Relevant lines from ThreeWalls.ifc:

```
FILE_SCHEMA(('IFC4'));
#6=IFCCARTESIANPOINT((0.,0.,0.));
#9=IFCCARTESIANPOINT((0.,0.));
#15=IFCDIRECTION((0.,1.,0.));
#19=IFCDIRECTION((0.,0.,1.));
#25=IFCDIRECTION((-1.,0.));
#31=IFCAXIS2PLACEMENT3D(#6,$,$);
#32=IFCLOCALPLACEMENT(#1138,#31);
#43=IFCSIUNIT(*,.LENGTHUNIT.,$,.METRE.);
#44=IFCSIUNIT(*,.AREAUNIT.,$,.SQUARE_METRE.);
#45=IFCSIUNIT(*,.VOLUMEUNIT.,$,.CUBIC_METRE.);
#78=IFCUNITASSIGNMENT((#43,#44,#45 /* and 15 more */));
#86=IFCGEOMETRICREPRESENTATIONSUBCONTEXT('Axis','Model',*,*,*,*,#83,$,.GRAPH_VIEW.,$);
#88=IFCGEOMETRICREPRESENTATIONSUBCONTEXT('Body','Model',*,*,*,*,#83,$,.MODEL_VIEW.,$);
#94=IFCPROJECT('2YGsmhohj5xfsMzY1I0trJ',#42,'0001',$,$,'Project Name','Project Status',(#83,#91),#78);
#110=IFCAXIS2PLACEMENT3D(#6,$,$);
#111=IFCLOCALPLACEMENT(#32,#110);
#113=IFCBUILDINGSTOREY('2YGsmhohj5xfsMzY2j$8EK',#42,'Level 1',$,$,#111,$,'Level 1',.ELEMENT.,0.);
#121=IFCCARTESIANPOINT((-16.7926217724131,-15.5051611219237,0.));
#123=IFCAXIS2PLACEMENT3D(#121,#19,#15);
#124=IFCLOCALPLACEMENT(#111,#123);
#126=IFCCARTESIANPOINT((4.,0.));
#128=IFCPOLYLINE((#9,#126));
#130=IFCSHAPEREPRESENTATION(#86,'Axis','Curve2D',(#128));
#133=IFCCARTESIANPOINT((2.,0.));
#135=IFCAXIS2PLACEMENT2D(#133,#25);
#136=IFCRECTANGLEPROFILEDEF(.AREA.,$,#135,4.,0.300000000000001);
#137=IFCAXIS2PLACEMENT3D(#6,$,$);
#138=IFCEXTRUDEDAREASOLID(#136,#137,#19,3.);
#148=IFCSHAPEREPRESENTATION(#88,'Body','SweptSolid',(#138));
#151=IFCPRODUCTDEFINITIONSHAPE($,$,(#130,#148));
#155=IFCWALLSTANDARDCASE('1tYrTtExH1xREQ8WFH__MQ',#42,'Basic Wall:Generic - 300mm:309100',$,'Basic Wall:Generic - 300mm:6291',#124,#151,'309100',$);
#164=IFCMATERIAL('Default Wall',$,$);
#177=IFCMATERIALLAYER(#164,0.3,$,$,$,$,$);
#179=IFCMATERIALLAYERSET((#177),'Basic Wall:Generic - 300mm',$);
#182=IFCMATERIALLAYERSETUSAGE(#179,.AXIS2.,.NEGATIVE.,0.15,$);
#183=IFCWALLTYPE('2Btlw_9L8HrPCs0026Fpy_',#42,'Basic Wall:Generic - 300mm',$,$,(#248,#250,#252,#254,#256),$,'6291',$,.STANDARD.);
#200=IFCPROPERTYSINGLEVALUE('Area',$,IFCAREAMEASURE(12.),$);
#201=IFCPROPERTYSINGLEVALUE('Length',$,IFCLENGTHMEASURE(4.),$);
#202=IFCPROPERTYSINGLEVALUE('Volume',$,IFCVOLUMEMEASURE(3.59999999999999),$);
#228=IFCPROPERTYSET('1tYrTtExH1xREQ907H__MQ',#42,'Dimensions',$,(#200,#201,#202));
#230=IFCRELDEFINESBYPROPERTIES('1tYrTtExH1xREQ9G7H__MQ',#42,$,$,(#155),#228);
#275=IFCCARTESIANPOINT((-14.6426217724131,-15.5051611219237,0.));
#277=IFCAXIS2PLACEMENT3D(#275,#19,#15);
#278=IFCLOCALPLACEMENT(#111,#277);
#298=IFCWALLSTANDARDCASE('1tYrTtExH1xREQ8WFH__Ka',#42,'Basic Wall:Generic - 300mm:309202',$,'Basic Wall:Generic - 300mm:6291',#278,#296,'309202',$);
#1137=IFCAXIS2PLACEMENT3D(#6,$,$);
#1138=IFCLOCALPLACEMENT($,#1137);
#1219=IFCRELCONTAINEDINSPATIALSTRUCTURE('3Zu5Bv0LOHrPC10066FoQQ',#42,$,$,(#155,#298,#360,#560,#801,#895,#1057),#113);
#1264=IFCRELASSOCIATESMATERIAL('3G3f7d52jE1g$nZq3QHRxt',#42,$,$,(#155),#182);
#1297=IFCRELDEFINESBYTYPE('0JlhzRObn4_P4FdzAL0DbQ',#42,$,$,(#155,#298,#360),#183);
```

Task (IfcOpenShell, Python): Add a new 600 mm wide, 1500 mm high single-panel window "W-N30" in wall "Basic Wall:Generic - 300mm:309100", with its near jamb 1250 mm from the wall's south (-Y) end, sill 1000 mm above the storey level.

```python
import numpy as np
import ifcopenshell
import ifcopenshell.api.feature
import ifcopenshell.api.geometry
import ifcopenshell.api.pset
import ifcopenshell.api.root
import ifcopenshell.api.spatial
import ifcopenshell.geom
import ifcopenshell.util.element
import ifcopenshell.util.placement
import ifcopenshell.util.representation
import ifcopenshell.util.shape
import ifcopenshell.util.unit

model = ifcopenshell.open("ThreeWalls.ifc")
unit_scale = ifcopenshell.util.unit.calculate_unit_scale(model)
area_scale = ifcopenshell.util.unit.calculate_unit_scale(model, "AREAUNIT")
volume_scale = ifcopenshell.util.unit.calculate_unit_scale(model, "VOLUMEUNIT")
settings = ifcopenshell.geom.settings()


def volume(element):
    """Net volume in cubic metres, openings subtracted."""
    shape = ifcopenshell.geom.create_shape(settings, element)
    return ifcopenshell.util.shape.get_volume(shape.geometry)


wall = model.by_guid("1tYrTtExH1xREQ8WFH__MQ")
storey = ifcopenshell.util.element.get_container(wall, ifc_class="IfcBuildingStorey")
context = ifcopenshell.util.representation.get_context(model, "Model", "Body", "MODEL_VIEW")
before = volume(wall)

width, height, from_end, sill = 0.6, 1.5, 1.25, 1  # metres

# The wall runs along its own X axis, and the end named is its -X end.
wall_shape = ifcopenshell.geom.create_shape(settings, wall)
x, y, z = ifcopenshell.util.shape.get_vertices(wall_shape.geometry).T
start = x.min() + from_end
face, thickness = float(y.min()), float(y.max() - y.min())
wall_matrix = ifcopenshell.util.placement.get_local_placement(wall.ObjectPlacement)
level = ifcopenshell.util.placement.get_local_placement(storey.ObjectPlacement)[2, 3]


def in_wall(x, y):
    """Placement at x, y metres in the wall's axes, at sill height."""
    matrix = wall_matrix.copy()
    matrix[:, 3] = wall_matrix @ np.array([x / unit_scale, y / unit_scale, 0.0, 1.0])
    matrix[2, 3] = level + sill / unit_scale
    return matrix


# Opening: a box that overshoots both wall faces by 50 mm.
opening = ifcopenshell.api.root.create_entity(model, ifc_class="IfcOpeningElement", predefined_type="OPENING")
box = ifcopenshell.api.geometry.add_wall_representation(
    model, context=context, length=width, height=height, thickness=thickness + 0.1
)
ifcopenshell.api.geometry.assign_representation(model, product=opening, representation=box)
ifcopenshell.api.geometry.edit_object_placement(model, product=opening, matrix=in_wall(start, face - 0.05), is_si=False)
ifcopenshell.api.feature.add_feature(model, feature=opening, element=wall)

window = ifcopenshell.api.root.create_entity(model, ifc_class="IfcWindow", name="W-N30", predefined_type="WINDOW")
window.OverallWidth, window.OverallHeight = width / unit_scale, height / unit_scale
window.PartitioningType = "SINGLE_PANEL"
body = ifcopenshell.api.geometry.add_window_representation(
    model,
    context=context,
    overall_width=window.OverallWidth,
    overall_height=window.OverallHeight,
    partition_type="SINGLE_PANEL",
)
ifcopenshell.api.geometry.assign_representation(model, product=window, representation=body)
ifcopenshell.api.spatial.assign_container(model, products=[window], relating_structure=storey)
ifcopenshell.api.feature.add_filling(model, opening=opening, element=window)

# Centre the window in the wall's thickness.
ifcopenshell.api.geometry.edit_object_placement(model, product=window, matrix=in_wall(start, face), is_si=False)
window_shape = ifcopenshell.geom.create_shape(settings, window)
depth = ifcopenshell.util.shape.get_vertices(window_shape.geometry)[:, 1]
offset = face + thickness / 2 - (depth.min() + depth.max()) / 2
ifcopenshell.api.geometry.edit_object_placement(model, product=window, matrix=in_wall(start, offset), is_si=False)

after = volume(wall)

# Update the wall's stored quantities.
pset = model.by_id(ifcopenshell.util.element.get_pset(wall, "Dimensions", should_inherit=False)["id"])
ifcopenshell.api.pset.edit_pset(model, pset=pset, properties={
    "Area": model.create_entity("IfcAreaMeasure", after / thickness / area_scale),
    "Volume": model.create_entity("IfcVolumeMeasure", after / volume_scale),
})

print(f"wall volume {before:.3f} -> {after:.3f} m3")

model.write("ThreeWalls_updated.ifc")
```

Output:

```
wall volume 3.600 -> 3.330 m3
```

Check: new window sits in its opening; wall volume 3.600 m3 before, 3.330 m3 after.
